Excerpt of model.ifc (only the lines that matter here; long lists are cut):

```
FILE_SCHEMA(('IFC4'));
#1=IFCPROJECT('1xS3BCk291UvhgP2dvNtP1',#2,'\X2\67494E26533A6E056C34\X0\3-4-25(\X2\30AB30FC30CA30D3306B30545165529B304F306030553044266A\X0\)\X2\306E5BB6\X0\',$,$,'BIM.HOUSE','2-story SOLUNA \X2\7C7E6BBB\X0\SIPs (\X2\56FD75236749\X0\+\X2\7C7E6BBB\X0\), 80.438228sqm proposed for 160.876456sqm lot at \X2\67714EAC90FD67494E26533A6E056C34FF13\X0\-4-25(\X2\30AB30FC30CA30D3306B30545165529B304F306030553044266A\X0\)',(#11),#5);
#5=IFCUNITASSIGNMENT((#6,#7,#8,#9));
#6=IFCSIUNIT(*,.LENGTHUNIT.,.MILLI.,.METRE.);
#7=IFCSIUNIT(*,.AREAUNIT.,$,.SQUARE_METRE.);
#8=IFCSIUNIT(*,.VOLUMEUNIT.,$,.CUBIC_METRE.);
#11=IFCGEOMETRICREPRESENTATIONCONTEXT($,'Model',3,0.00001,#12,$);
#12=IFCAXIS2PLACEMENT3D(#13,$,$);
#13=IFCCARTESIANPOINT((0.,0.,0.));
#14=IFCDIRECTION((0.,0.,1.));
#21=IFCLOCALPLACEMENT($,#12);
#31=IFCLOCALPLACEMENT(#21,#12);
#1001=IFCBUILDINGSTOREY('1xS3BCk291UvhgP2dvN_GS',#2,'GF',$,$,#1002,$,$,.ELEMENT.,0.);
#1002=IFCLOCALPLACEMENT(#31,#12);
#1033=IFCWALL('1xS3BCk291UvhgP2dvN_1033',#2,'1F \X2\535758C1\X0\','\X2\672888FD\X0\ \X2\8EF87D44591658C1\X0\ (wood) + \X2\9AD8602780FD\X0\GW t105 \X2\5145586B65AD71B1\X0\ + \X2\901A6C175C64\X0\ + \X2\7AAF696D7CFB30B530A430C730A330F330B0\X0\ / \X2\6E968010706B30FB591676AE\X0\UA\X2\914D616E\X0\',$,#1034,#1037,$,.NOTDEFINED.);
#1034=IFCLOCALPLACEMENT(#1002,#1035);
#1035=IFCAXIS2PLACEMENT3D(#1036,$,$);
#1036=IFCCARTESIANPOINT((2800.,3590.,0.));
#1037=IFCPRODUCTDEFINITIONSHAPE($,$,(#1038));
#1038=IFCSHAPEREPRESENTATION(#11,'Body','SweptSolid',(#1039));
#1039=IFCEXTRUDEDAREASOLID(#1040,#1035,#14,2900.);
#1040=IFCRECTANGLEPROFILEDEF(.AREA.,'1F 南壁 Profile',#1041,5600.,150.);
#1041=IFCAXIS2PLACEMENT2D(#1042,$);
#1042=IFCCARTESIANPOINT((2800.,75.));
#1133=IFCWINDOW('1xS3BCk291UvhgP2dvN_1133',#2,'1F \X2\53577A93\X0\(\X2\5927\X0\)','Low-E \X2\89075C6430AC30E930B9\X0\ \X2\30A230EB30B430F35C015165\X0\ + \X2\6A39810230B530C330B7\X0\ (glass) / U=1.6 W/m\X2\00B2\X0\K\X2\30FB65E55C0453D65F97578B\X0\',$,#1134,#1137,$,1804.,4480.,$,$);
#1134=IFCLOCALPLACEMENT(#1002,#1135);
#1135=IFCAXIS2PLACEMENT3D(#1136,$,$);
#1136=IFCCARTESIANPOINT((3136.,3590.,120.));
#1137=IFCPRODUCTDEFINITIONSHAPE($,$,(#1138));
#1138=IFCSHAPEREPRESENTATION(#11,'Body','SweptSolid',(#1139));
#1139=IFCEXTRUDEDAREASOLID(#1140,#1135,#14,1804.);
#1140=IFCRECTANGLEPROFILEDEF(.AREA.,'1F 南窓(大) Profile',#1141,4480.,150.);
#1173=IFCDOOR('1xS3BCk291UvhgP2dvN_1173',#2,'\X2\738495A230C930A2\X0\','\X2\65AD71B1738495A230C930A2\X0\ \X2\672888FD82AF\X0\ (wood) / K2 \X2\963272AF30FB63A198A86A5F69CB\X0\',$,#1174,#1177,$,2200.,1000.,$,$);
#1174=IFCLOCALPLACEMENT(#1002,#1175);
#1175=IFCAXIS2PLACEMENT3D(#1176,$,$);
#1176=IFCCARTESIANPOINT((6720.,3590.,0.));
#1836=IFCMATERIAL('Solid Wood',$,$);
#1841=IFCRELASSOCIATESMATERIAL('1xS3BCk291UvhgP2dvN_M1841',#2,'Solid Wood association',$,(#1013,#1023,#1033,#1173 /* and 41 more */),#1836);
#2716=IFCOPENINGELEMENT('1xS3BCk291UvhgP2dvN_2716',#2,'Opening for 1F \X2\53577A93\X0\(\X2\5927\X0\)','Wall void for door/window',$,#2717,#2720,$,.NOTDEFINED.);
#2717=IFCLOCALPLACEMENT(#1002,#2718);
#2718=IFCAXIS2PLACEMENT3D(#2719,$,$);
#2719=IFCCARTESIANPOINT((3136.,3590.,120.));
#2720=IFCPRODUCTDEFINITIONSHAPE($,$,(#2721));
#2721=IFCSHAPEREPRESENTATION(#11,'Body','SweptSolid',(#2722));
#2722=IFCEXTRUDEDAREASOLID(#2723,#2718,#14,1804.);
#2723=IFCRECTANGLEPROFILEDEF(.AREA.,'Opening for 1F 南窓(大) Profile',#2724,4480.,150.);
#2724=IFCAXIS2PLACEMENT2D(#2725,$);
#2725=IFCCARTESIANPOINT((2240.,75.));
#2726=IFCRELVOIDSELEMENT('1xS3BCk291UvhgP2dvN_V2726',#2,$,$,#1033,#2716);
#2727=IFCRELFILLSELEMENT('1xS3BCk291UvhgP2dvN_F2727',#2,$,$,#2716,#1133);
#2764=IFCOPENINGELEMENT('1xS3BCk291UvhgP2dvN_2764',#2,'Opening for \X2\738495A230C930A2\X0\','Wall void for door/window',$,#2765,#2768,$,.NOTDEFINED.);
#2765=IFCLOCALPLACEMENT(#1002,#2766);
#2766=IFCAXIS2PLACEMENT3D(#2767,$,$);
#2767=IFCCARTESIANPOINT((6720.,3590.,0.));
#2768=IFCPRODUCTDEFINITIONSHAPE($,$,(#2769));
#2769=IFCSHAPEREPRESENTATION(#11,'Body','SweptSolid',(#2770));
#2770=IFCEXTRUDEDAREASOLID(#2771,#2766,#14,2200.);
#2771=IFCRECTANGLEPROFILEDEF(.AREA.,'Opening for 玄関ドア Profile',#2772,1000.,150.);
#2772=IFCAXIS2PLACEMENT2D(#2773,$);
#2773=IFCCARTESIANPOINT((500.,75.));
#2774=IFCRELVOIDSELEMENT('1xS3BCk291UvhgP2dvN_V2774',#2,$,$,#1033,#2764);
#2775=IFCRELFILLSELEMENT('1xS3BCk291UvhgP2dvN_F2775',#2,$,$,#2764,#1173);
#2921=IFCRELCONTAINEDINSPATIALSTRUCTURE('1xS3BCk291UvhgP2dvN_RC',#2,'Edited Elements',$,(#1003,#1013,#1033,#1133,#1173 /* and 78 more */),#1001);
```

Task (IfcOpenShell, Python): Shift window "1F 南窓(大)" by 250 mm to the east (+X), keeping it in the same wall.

```python
import ifcopenshell
import ifcopenshell.api.geometry
import ifcopenshell.util.placement
import ifcopenshell.util.unit

model = ifcopenshell.open("model.ifc")
unit_scale = ifcopenshell.util.unit.calculate_unit_scale(model)

window = model.by_guid("1xS3BCk291UvhgP2dvN_1133")
opening = window.FillsVoids[0].RelatingOpeningElement
wall = opening.VoidsElements[0].RelatingBuildingElement

wall_matrix = ifcopenshell.util.placement.get_local_placement(wall.ObjectPlacement)
shift = wall_matrix[:3, 0] * 0.25 / unit_scale
before = ifcopenshell.util.placement.get_local_placement(window.ObjectPlacement)[:3, 3].copy()

# The window is not placed relative to its opening, so move both.
for product in (opening, window):
    matrix = ifcopenshell.util.placement.get_local_placement(product.ObjectPlacement)
    matrix[:3, 3] += shift
    ifcopenshell.api.geometry.edit_object_placement(model, product=product, matrix=matrix, is_si=False)

after = ifcopenshell.util.placement.get_local_placement(window.ObjectPlacement)[:3, 3]
print("window moved by", (after - before).round(3) + 0.0)

model.write("model_updated.ifc")
```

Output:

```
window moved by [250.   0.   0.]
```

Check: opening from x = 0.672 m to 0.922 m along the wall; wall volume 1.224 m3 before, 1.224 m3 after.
